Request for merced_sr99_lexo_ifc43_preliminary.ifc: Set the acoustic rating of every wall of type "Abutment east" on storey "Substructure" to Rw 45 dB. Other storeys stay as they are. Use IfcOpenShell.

First a look at what the model holds.

```python
import ifcopenshell
import ifcopenshell.util.element

model = ifcopenshell.open("merced_sr99_lexo_ifc43_preliminary.ifc")
print(model.schema)
storey = next(s for s in model.by_type("IfcBuildingStorey") if s.Name == "Substructure")
walls = [e for e in ifcopenshell.util.element.get_decomposition(storey) if e.is_a("IfcWall")]
seen = {}
for e in walls:
    element_type = ifcopenshell.util.element.get_type(e)
    key = (element_type.Name if element_type != e and element_type else None, ifcopenshell.util.element.get_pset(e, "Pset_WallCommon", "AcousticRating"))
    seen[key] = seen.get(key, 0) + 1
for (name, value), count in sorted(seen.items(), key=str):
    print(count, "x", name, "|", value)
```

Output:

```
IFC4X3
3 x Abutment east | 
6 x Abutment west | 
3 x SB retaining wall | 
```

```python
import ifcopenshell
import ifcopenshell.api.pset
import ifcopenshell.util.element

model = ifcopenshell.open("merced_sr99_lexo_ifc43_preliminary.ifc")

storey = next(s for s in model.by_type("IfcBuildingStorey") if s.Name == "Substructure")
walls = [e for e in ifcopenshell.util.element.get_decomposition(storey) if e.is_a("IfcWall")]

count = 0
for e in walls:
    element_type = ifcopenshell.util.element.get_type(e)
    if element_type in (None, e) or element_type.Name != "Abutment east":
        continue
    # add_pset returns the element's existing set when there is one.
    pset = ifcopenshell.api.pset.add_pset(model, product=e, name="Pset_WallCommon")
    ifcopenshell.api.pset.edit_pset(model, pset=pset, properties={"AcousticRating": "Rw 45 dB"})
    count += 1

print(count, "walls updated")

model.write("merced_sr99_lexo_ifc43_preliminary_edited.ifc")
```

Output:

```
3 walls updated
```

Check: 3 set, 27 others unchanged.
